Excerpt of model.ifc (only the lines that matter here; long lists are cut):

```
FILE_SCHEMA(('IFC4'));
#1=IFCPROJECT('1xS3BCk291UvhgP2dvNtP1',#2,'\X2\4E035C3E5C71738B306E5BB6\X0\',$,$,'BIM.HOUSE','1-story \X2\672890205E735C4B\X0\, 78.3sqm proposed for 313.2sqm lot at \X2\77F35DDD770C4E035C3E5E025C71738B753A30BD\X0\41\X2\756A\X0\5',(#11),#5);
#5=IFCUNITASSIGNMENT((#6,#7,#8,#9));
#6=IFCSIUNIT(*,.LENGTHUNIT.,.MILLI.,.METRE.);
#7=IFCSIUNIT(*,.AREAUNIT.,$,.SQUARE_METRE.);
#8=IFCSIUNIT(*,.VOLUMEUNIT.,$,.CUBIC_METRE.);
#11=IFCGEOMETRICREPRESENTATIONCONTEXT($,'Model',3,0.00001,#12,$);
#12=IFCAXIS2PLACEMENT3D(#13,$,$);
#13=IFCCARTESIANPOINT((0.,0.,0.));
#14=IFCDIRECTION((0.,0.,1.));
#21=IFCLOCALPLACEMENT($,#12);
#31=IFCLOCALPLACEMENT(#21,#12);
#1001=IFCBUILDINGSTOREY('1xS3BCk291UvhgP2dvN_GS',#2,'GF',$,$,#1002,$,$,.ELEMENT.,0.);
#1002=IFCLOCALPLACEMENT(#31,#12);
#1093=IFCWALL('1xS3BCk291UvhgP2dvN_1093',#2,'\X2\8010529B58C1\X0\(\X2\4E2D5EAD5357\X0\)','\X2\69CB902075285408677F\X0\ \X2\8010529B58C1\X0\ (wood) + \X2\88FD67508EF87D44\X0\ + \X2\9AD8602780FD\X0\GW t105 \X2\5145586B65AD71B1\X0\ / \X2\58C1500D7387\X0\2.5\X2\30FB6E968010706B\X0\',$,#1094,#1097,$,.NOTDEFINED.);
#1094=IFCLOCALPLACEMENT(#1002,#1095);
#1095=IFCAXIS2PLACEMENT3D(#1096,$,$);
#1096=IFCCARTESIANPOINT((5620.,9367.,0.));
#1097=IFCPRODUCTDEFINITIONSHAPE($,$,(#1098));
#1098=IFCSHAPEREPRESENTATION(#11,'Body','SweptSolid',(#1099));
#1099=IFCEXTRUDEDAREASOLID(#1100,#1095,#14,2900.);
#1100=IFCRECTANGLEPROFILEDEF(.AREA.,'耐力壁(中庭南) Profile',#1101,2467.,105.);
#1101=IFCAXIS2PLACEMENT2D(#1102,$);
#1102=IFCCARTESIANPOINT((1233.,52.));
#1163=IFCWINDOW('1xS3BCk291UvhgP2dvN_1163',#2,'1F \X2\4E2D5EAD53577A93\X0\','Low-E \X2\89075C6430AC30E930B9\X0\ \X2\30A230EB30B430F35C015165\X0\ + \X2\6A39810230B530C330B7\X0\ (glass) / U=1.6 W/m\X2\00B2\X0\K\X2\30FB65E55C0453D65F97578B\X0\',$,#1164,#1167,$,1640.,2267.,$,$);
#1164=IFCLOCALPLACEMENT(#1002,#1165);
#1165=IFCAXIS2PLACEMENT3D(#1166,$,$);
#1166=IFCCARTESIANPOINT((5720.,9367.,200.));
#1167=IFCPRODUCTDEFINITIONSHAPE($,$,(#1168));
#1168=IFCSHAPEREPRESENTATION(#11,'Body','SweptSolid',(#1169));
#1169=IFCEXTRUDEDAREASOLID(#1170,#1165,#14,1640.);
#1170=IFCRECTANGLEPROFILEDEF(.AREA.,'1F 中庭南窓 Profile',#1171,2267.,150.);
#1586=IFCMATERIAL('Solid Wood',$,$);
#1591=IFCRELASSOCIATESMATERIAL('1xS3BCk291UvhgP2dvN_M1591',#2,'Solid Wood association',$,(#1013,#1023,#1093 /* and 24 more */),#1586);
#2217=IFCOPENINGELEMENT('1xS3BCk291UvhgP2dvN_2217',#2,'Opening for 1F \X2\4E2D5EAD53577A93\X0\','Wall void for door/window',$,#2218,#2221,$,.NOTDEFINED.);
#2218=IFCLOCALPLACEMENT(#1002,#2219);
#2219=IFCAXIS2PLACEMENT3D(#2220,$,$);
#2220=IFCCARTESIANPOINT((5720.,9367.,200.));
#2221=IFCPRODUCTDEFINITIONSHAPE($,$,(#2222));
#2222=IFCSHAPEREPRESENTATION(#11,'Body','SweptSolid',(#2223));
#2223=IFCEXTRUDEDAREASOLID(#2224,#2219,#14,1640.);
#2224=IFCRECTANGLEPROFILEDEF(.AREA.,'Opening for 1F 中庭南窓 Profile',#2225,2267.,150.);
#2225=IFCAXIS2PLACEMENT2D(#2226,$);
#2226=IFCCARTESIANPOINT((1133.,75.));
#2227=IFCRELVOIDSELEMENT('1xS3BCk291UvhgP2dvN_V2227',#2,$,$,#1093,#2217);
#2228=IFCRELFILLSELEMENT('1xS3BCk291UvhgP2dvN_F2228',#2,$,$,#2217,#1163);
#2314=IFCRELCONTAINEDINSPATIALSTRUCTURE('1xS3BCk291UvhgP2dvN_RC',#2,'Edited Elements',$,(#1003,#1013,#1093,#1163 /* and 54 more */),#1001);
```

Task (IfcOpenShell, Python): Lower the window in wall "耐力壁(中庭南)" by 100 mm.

```python
import numpy as np
import ifcopenshell
import ifcopenshell.api.geometry
import ifcopenshell.util.placement
import ifcopenshell.util.unit

model = ifcopenshell.open("model.ifc")
unit_scale = ifcopenshell.util.unit.calculate_unit_scale(model)

window = model.by_guid("1xS3BCk291UvhgP2dvN_1163")
opening = window.FillsVoids[0].RelatingOpeningElement
dz = -0.1 / unit_scale

shift = np.array([0.0, 0.0, dz])
# The window is not placed relative to its opening, so move both.
for product in (opening, window):
    matrix = ifcopenshell.util.placement.get_local_placement(product.ObjectPlacement)
    matrix[:3, 3] += shift
    ifcopenshell.api.geometry.edit_object_placement(model, product=product, matrix=matrix, is_si=False)

print(f"moved by {dz * unit_scale:+.3f} m")

model.write("model_rev.ifc")
```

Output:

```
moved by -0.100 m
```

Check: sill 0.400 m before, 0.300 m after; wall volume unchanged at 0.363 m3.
